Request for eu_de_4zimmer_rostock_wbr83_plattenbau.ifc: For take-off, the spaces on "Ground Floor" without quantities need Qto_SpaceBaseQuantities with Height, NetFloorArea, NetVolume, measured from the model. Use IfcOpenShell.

First a look at what the model holds.

```python
import ifcopenshell
import ifcopenshell.util.element
import ifcopenshell.util.unit

model = ifcopenshell.open("eu_de_4zimmer_rostock_wbr83_plattenbau.ifc")
print(model.schema)
for unit_type in ("LENGTHUNIT", "AREAUNIT", "VOLUMEUNIT"):
    print(unit_type, ifcopenshell.util.unit.calculate_unit_scale(model, unit_type))
storey = next(s for s in model.by_type("IfcBuildingStorey") if s.Name == "Ground Floor")
spaces = [e for e in ifcopenshell.util.element.get_decomposition(storey) if e.is_a("IfcSpace")]
for e in sorted(spaces, key=lambda e: e.id()):
    print(e.id(), e.is_a(), e.Name, list(ifcopenshell.util.element.get_psets(e, qtos_only=True)), sep=" | ")
```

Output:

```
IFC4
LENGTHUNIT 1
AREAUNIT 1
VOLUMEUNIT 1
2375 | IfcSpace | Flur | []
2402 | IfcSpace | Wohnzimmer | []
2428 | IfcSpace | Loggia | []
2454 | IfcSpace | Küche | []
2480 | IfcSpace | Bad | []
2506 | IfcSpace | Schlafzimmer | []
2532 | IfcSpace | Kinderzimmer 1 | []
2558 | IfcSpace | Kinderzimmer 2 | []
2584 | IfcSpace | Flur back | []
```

```python
import ifcopenshell
import ifcopenshell.api.pset
import ifcopenshell.geom
import ifcopenshell.util.element
import ifcopenshell.util.shape
import ifcopenshell.util.unit

model = ifcopenshell.open("eu_de_4zimmer_rostock_wbr83_plattenbau.ifc")
unit_scale = ifcopenshell.util.unit.calculate_unit_scale(model)
area_scale = ifcopenshell.util.unit.calculate_unit_scale(model, "AREAUNIT")
volume_scale = ifcopenshell.util.unit.calculate_unit_scale(model, "VOLUMEUNIT")
settings = ifcopenshell.geom.settings()

storey = next(s for s in model.by_type("IfcBuildingStorey") if s.Name == "Ground Floor")
spaces = [e for e in ifcopenshell.util.element.get_decomposition(storey) if e.is_a("IfcSpace")]

for e in sorted(spaces, key=lambda e: e.id()):
    if ifcopenshell.util.element.get_psets(e, qtos_only=True, should_inherit=False):
        continue
    # Geometry comes back in metres, in the element's own axes.
    shape = ifcopenshell.geom.create_shape(settings, e)
    values = {
        "Height": ifcopenshell.util.shape.get_z(shape.geometry) / unit_scale,
        "NetFloorArea": ifcopenshell.util.shape.get_footprint_area(shape.geometry) / area_scale,
        "NetVolume": ifcopenshell.util.shape.get_volume(shape.geometry) / volume_scale,
    }
    qto = ifcopenshell.api.pset.add_qto(model, product=e, name="Qto_SpaceBaseQuantities")
    ifcopenshell.api.pset.edit_qto(model, qto=qto, properties=values)
    print(e.id(), {k: round(v, 3) for k, v in values.items()})

model.write("eu_de_4zimmer_rostock_wbr83_plattenbau_v2.ifc")
```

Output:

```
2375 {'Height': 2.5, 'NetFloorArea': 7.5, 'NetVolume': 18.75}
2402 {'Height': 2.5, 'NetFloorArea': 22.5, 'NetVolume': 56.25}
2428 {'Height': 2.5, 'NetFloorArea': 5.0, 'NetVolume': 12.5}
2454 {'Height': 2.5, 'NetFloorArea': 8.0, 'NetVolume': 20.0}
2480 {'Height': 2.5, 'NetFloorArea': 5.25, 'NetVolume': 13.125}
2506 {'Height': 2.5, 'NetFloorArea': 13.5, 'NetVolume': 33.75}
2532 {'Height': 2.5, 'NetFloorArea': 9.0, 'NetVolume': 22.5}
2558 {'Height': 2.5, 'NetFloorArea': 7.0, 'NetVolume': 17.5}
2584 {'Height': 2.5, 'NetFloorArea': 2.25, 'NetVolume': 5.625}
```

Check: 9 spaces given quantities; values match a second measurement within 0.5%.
